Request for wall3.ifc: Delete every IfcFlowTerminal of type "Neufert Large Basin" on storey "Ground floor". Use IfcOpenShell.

First a look at what the model holds.

```python
import ifcopenshell
import ifcopenshell.util.element

model = ifcopenshell.open("wall3.ifc")
print(model.schema)
storey = next(s for s in model.by_type("IfcBuildingStorey") if s.Name == "Ground floor")
terminals = [e for e in ifcopenshell.util.element.get_decomposition(storey) if e.is_a("IfcFlowTerminal")]
seen = {}
for e in terminals:
    element_type = ifcopenshell.util.element.get_type(e)
    name = element_type.Name if element_type not in (None, e) else None
    seen[name] = seen.get(name, 0) + 1
for name, count in sorted(seen.items(), key=str):
    print(count, "x", name)
```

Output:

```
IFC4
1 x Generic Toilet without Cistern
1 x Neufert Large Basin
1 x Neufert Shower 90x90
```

```python
import ifcopenshell
import ifcopenshell.api.root
import ifcopenshell.util.element

model = ifcopenshell.open("wall3.ifc")

storey = next(s for s in model.by_type("IfcBuildingStorey") if s.Name == "Ground floor")
terminals = [e for e in ifcopenshell.util.element.get_decomposition(storey) if e.is_a("IfcFlowTerminal")]
targets = [e for e in terminals if (t := ifcopenshell.util.element.get_type(e)) not in (None, e) and t.Name == "Neufert Large Basin"]

for e in targets:
    ifcopenshell.api.root.remove_product(model, product=e)
print(len(targets), "removed")

model.write("wall3-out.ifc")
```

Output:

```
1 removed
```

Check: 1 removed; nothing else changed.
